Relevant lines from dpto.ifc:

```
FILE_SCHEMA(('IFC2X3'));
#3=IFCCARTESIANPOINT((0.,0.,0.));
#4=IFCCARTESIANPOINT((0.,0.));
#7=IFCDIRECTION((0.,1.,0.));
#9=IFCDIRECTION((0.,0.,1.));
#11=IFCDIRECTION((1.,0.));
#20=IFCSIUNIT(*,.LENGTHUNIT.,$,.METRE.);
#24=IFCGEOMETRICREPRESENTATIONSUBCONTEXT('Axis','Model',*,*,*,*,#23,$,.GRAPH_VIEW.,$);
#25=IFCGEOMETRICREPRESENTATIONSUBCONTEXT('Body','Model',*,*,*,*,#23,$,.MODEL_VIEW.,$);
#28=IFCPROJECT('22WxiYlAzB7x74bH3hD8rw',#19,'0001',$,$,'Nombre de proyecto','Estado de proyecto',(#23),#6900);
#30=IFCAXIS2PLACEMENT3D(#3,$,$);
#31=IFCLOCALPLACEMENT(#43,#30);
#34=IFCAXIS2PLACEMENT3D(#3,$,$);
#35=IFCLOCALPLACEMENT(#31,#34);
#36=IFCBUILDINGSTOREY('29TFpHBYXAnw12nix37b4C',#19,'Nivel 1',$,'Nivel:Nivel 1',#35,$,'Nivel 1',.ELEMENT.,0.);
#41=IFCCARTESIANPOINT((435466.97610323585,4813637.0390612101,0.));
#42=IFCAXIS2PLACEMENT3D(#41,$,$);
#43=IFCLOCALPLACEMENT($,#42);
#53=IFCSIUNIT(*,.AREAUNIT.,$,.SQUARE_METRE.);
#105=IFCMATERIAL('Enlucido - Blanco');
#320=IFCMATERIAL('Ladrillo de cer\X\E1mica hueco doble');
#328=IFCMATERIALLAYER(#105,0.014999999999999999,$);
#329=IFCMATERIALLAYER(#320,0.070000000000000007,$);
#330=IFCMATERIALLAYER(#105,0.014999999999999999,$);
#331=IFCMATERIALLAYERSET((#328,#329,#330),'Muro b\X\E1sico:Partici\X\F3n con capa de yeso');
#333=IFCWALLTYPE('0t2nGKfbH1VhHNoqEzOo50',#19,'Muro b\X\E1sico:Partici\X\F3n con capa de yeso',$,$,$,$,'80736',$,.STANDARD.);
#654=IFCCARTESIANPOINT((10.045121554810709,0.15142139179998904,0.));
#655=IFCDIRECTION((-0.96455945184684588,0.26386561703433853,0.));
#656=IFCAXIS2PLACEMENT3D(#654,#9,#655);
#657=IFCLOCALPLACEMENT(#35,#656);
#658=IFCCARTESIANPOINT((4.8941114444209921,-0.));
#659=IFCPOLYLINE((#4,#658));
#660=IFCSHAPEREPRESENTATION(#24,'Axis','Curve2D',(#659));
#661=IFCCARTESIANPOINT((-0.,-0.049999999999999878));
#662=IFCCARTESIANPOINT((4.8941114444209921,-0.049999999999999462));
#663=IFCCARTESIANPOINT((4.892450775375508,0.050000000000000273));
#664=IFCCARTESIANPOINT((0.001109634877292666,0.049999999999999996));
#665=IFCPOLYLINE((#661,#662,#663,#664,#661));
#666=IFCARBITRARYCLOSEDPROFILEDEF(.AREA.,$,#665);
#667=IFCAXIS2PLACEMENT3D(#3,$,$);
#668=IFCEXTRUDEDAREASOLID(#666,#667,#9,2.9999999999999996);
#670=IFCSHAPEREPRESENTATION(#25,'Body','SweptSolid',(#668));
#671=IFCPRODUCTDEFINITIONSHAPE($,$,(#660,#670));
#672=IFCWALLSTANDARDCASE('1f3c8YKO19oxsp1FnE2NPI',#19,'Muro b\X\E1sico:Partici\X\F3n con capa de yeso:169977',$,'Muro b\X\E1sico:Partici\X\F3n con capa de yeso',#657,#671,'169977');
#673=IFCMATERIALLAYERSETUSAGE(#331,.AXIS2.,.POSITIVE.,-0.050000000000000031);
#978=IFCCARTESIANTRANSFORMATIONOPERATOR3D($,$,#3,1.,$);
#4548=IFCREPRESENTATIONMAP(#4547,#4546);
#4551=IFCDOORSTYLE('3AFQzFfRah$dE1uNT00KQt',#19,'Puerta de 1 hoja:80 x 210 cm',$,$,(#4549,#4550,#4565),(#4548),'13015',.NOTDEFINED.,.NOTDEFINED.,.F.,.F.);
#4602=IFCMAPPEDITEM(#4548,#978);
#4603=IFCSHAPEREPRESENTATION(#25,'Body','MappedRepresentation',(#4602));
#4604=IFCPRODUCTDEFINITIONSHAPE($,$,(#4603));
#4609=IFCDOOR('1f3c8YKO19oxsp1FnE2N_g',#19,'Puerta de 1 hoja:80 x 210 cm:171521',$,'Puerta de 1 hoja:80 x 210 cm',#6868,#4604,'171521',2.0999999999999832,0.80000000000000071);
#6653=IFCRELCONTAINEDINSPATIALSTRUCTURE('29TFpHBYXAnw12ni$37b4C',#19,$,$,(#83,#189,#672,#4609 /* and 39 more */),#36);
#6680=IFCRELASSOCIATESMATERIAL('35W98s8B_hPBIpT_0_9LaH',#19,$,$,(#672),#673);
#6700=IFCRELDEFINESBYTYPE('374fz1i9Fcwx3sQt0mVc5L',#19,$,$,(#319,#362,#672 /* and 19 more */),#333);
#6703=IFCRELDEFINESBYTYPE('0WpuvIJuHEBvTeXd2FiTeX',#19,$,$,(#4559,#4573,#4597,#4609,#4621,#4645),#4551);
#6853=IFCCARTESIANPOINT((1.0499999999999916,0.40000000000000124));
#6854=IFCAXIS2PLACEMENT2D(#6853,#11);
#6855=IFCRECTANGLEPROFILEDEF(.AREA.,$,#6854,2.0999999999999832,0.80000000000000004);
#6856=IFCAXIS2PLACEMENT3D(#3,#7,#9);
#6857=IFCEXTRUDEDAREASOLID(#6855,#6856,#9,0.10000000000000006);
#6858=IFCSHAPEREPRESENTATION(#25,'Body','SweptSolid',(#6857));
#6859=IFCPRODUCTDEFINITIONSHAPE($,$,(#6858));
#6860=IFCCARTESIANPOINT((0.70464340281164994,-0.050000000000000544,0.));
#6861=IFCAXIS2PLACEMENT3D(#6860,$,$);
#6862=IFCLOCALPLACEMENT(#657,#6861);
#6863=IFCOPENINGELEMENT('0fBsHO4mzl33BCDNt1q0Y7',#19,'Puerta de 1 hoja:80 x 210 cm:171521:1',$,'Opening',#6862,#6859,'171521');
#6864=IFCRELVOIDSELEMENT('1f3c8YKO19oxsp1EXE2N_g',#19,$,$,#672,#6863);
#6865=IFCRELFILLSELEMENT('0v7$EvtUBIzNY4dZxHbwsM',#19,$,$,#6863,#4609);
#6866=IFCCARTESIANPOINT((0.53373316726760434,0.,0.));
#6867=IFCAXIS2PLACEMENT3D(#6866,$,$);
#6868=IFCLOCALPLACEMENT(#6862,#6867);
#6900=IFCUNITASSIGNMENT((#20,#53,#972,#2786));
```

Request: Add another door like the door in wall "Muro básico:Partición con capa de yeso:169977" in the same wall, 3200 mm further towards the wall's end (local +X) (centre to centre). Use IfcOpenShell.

```python
import ifcopenshell
import ifcopenshell.api.feature
import ifcopenshell.api.geometry
import ifcopenshell.api.root
import ifcopenshell.geom
import ifcopenshell.util.element
import ifcopenshell.util.placement
import ifcopenshell.util.shape

model = ifcopenshell.open("dpto.ifc")
settings = ifcopenshell.geom.settings()


def volume(element):
    """Net volume in cubic metres, openings subtracted."""
    shape = ifcopenshell.geom.create_shape(settings, element)
    return ifcopenshell.util.shape.get_volume(shape.geometry)


def reuse_history(source, copy):
    """copy_class also copies each property set's owner history, people and application; keep the originals."""
    for rel in copy.IsDefinedBy:
        if rel.is_a("IfcRelDefinesByProperties") and (history := rel.RelatingPropertyDefinition.OwnerHistory):
            rel.RelatingPropertyDefinition.OwnerHistory = source.OwnerHistory
            ifcopenshell.util.element.remove_deep2(model, history)


door = model.by_id(4609)
opening = door.FillsVoids[0].RelatingOpeningElement
wall = opening.VoidsElements[0].RelatingBuildingElement
before = volume(wall)
shift = ifcopenshell.util.placement.get_local_placement(wall.ObjectPlacement)[:3, 0] * 3.2

# copy_class copies the void relationship, type, container and properties, but no geometry.
new_opening = ifcopenshell.api.root.copy_class(model, product=opening)
new_opening.Representation = ifcopenshell.util.element.copy_deep(
    model, opening.Representation, exclude=["IfcGeometricRepresentationContext", "IfcRepresentationMap"]
)
new_opening.Name = "Puerta de 1 hoja:80 x 210 cm"
new_opening.Tag = None
new_door = ifcopenshell.api.root.copy_class(model, product=door)
new_door.Representation = ifcopenshell.util.element.copy_deep(
    model, door.Representation, exclude=["IfcGeometricRepresentationContext", "IfcRepresentationMap"]
)
new_door.Name = "Puerta de 1 hoja:80 x 210 cm"
new_door.Tag = None
reuse_history(door, new_door)
fills = ifcopenshell.api.feature.add_filling(model, opening=new_opening, element=new_door)
fills.OwnerHistory = new_door.OwnerHistory  # required in IFC2X3

for old, new in ((opening, new_opening), (door, new_door)):
    matrix = ifcopenshell.util.placement.get_local_placement(old.ObjectPlacement)
    matrix[:3, 3] += shift
    ifcopenshell.api.geometry.edit_object_placement(model, product=new, matrix=matrix, is_si=False)

after = volume(wall)

print(f"wall volume {before:.3f} -> {after:.3f} m3")

model.write("dpto_rev.ifc")
```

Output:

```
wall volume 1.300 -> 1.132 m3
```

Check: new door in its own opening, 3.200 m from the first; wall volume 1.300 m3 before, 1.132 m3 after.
